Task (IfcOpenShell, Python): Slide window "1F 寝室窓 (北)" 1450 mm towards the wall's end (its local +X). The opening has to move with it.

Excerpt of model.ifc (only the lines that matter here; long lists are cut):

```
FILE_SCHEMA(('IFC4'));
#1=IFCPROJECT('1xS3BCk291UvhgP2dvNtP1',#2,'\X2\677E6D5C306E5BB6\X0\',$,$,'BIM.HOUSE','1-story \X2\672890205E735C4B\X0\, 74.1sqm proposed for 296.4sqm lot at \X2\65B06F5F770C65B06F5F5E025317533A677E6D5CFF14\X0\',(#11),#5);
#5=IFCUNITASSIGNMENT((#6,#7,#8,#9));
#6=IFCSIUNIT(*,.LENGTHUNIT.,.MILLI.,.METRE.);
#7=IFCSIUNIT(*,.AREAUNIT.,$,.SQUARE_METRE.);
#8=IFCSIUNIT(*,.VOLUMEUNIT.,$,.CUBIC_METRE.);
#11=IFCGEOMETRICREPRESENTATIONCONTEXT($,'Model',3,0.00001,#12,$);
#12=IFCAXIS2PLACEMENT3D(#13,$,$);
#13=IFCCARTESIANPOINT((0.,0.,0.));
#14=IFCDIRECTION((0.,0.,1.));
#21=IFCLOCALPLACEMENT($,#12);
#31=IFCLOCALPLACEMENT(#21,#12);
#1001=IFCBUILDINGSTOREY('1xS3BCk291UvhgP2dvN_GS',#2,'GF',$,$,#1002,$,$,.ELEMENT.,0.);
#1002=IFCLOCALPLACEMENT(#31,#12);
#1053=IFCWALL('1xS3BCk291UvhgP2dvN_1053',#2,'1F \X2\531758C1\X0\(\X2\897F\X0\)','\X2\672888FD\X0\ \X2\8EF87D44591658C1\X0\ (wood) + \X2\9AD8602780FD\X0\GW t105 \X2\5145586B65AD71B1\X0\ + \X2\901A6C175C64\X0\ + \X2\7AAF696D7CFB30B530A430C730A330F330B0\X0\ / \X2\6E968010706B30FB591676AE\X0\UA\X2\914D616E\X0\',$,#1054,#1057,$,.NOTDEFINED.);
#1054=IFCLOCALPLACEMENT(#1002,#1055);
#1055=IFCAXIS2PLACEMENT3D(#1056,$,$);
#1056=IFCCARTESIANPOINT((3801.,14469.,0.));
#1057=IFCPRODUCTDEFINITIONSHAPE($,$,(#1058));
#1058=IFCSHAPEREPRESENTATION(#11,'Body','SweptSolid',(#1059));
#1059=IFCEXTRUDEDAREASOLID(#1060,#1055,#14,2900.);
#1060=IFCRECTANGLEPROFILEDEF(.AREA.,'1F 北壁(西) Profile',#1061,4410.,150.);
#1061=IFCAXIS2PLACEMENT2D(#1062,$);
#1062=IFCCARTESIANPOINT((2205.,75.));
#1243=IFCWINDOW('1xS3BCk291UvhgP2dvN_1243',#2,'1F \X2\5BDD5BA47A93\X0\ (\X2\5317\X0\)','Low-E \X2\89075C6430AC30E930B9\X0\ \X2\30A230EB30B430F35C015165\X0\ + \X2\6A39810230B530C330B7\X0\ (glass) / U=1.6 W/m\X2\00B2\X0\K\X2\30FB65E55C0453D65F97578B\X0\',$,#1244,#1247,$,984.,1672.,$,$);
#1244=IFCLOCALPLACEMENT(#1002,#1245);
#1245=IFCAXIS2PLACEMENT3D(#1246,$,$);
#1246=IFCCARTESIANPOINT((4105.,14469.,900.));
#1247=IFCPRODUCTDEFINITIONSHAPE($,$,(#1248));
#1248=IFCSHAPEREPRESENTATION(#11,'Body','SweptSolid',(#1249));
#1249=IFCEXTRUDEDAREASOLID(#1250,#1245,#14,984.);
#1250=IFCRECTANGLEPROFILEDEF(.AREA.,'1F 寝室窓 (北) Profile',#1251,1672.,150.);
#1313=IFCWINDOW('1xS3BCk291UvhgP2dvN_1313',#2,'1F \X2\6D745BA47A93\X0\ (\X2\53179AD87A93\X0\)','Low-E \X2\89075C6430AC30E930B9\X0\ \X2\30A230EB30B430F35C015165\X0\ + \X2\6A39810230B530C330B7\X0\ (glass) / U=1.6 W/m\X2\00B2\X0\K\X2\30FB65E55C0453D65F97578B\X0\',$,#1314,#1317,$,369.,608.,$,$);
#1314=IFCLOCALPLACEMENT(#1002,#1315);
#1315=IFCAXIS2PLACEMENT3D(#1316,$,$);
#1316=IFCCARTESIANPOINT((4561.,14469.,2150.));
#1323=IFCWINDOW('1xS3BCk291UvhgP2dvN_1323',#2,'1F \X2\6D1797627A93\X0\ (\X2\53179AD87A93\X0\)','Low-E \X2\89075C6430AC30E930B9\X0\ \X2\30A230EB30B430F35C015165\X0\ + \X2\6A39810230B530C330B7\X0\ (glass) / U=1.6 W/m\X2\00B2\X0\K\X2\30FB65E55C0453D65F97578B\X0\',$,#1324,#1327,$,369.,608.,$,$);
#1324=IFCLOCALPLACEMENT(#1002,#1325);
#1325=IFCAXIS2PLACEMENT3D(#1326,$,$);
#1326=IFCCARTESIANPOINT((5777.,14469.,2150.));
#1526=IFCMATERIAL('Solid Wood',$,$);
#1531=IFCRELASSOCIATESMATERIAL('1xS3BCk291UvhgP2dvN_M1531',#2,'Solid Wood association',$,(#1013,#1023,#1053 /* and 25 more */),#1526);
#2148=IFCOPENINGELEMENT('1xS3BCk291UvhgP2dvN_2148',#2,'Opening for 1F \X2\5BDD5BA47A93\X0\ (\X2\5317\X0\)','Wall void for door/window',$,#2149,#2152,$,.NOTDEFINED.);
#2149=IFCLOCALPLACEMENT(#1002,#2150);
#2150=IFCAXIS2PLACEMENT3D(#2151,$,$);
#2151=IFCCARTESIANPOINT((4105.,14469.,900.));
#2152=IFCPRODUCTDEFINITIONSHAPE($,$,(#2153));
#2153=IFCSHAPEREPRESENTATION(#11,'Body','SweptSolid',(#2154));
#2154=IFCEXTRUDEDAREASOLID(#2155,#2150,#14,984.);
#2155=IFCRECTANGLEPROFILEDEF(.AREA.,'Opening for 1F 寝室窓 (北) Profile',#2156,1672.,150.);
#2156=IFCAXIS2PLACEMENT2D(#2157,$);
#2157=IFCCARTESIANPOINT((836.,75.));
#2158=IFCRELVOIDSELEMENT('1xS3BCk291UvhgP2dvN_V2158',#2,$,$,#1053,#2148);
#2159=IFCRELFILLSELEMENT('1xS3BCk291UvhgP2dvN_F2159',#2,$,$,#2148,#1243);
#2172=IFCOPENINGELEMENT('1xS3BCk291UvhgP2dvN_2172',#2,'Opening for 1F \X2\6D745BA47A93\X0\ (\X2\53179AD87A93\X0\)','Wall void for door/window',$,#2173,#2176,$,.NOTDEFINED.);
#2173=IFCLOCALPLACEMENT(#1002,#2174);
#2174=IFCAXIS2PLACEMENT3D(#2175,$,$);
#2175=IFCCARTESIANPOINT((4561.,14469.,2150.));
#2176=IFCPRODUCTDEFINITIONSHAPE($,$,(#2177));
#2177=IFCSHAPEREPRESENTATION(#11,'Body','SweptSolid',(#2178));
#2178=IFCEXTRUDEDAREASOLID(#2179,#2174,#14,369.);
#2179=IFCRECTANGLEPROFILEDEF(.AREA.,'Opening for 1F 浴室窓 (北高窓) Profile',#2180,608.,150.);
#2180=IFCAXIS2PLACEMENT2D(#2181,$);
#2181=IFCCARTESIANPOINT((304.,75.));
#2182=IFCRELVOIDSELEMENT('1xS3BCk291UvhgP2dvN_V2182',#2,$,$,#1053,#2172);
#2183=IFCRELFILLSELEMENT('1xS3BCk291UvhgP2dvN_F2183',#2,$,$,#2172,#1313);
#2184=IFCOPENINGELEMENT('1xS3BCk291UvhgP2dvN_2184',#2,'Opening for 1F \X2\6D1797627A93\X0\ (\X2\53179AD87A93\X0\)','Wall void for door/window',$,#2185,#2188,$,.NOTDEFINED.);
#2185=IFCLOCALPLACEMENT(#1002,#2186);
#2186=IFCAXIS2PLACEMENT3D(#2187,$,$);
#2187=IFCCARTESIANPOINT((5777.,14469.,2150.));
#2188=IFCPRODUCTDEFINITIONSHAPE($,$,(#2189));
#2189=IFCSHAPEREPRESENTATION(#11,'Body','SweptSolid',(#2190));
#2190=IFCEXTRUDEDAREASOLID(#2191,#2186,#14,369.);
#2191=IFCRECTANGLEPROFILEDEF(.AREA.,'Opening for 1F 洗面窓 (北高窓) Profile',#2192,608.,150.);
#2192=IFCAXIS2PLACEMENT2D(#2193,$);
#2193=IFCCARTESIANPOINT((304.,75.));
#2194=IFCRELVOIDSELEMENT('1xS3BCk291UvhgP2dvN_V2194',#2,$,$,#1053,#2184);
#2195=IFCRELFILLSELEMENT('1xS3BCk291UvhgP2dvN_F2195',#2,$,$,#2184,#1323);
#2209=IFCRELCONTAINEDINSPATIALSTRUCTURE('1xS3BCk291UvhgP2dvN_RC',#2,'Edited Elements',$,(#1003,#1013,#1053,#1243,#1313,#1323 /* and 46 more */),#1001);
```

```python
import ifcopenshell
import ifcopenshell.api.geometry
import ifcopenshell.util.placement

model = ifcopenshell.open("model.ifc")

window = model.by_id(1243)
opening = window.FillsVoids[0].RelatingOpeningElement
wall = opening.VoidsElements[0].RelatingBuildingElement

wall_matrix = ifcopenshell.util.placement.get_local_placement(wall.ObjectPlacement)
shift = wall_matrix[:3, 0] * 1450.0
before = ifcopenshell.util.placement.get_local_placement(window.ObjectPlacement)[:3, 3].copy()

# The window is not placed relative to its opening, so move both.
for product in (opening, window):
    matrix = ifcopenshell.util.placement.get_local_placement(product.ObjectPlacement)
    matrix[:3, 3] += shift
    ifcopenshell.api.geometry.edit_object_placement(model, product=product, matrix=matrix, is_si=False)

after = ifcopenshell.util.placement.get_local_placement(window.ObjectPlacement)[:3, 3]
print("window moved by", (after - before).round(3) + 0.0)

model.write("model_rev.ifc")
```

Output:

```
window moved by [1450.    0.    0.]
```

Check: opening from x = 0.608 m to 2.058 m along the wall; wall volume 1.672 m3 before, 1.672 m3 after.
